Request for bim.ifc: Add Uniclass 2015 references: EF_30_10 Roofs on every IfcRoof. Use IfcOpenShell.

First a look at what the model holds.

```python
import ifcopenshell

model = ifcopenshell.open("bim.ifc")
print(model.schema)
print("classifications:", [c.Name for c in model.by_type("IfcClassification")])
for ifc_class in ("IfcDoor", "IfcRoof", "IfcStair", "IfcWall", "IfcWindow"):
    print(ifc_class, len(model.by_type(ifc_class)))
```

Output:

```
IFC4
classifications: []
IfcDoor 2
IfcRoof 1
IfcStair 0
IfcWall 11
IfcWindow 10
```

```python
import ifcopenshell
import ifcopenshell.api.classification

model = ifcopenshell.open("bim.ifc")

system = ifcopenshell.api.classification.add_classification(model, classification="Uniclass 2015")

codes = {
    "IfcRoof": ("EF_30_10", "Roofs"),
}
for ifc_class, (code, name) in codes.items():
    products = model.by_type(ifc_class)
    ifcopenshell.api.classification.add_reference(
        model, products=products, classification=system, identification=code, name=name
    )
    print(code, len(products))

model.write("bim-out.ifc")
```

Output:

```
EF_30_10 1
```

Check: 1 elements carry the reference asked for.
